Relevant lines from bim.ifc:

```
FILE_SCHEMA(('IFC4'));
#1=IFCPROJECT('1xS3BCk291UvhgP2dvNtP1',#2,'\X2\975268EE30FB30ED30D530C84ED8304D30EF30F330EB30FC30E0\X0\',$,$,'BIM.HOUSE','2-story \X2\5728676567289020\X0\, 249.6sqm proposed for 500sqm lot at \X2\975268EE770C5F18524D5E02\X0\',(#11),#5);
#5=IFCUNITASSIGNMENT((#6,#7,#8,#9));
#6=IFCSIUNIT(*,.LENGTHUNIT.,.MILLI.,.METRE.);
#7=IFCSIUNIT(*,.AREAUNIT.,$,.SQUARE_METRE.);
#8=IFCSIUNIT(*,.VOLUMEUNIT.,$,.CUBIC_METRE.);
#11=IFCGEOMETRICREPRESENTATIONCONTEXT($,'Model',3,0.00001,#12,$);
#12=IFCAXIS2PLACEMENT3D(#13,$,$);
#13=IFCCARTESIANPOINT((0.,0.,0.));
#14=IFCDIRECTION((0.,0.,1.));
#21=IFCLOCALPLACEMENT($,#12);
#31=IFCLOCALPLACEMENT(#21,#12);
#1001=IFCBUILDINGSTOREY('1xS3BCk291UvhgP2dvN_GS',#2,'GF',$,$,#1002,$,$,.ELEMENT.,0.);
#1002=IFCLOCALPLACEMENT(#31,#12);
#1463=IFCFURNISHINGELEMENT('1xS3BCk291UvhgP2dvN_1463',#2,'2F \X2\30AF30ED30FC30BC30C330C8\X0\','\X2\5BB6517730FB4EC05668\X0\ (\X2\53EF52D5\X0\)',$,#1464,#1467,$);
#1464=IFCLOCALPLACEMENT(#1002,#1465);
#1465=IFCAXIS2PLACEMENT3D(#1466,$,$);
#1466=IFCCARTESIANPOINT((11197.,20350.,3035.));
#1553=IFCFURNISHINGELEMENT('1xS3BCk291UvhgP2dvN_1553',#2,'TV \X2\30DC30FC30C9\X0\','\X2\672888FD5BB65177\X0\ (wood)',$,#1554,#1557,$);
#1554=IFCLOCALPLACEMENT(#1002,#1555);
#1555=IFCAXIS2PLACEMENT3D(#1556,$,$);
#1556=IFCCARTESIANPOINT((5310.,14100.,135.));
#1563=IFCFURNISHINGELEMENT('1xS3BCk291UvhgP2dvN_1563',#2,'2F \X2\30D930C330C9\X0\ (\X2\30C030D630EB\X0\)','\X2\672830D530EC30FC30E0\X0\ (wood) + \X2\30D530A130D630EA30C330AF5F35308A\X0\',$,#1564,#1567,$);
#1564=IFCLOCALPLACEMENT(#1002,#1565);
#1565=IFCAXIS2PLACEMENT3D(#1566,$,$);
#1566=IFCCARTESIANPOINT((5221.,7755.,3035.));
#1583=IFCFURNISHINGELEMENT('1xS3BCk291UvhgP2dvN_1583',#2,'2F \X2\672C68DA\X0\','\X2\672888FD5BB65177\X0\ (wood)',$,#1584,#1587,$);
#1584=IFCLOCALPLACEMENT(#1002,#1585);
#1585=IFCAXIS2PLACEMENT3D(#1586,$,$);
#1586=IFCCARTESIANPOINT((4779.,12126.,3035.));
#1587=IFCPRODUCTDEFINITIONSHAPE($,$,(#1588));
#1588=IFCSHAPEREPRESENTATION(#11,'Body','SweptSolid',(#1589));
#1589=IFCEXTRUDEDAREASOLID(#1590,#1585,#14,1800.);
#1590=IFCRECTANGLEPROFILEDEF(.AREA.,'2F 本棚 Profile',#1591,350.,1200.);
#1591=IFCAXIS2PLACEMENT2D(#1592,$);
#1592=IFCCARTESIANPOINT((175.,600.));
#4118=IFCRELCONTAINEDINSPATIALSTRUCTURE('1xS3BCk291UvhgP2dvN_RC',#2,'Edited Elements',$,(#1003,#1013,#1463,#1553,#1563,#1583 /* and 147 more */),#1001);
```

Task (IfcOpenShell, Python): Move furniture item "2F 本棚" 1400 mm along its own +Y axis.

```python
import ifcopenshell
import ifcopenshell.api.geometry
import ifcopenshell.util.placement
import ifcopenshell.util.unit

model = ifcopenshell.open("bim.ifc")
unit_scale = ifcopenshell.util.unit.calculate_unit_scale(model)

item = model.by_id(1583)
matrix = ifcopenshell.util.placement.get_local_placement(item.ObjectPlacement)
matrix[:3, 3] += matrix[:3, 1] * 1.4 / unit_scale
ifcopenshell.api.geometry.edit_object_placement(model, product=item, matrix=matrix, is_si=False)

print(ifcopenshell.util.placement.get_local_placement(item.ObjectPlacement).round(3) + 0.0)

model.write("bim_v2.ifc")
```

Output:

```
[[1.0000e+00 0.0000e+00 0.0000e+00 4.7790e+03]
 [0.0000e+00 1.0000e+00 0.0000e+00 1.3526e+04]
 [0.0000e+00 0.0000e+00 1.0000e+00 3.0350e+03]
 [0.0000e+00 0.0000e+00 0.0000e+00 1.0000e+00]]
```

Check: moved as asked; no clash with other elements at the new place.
